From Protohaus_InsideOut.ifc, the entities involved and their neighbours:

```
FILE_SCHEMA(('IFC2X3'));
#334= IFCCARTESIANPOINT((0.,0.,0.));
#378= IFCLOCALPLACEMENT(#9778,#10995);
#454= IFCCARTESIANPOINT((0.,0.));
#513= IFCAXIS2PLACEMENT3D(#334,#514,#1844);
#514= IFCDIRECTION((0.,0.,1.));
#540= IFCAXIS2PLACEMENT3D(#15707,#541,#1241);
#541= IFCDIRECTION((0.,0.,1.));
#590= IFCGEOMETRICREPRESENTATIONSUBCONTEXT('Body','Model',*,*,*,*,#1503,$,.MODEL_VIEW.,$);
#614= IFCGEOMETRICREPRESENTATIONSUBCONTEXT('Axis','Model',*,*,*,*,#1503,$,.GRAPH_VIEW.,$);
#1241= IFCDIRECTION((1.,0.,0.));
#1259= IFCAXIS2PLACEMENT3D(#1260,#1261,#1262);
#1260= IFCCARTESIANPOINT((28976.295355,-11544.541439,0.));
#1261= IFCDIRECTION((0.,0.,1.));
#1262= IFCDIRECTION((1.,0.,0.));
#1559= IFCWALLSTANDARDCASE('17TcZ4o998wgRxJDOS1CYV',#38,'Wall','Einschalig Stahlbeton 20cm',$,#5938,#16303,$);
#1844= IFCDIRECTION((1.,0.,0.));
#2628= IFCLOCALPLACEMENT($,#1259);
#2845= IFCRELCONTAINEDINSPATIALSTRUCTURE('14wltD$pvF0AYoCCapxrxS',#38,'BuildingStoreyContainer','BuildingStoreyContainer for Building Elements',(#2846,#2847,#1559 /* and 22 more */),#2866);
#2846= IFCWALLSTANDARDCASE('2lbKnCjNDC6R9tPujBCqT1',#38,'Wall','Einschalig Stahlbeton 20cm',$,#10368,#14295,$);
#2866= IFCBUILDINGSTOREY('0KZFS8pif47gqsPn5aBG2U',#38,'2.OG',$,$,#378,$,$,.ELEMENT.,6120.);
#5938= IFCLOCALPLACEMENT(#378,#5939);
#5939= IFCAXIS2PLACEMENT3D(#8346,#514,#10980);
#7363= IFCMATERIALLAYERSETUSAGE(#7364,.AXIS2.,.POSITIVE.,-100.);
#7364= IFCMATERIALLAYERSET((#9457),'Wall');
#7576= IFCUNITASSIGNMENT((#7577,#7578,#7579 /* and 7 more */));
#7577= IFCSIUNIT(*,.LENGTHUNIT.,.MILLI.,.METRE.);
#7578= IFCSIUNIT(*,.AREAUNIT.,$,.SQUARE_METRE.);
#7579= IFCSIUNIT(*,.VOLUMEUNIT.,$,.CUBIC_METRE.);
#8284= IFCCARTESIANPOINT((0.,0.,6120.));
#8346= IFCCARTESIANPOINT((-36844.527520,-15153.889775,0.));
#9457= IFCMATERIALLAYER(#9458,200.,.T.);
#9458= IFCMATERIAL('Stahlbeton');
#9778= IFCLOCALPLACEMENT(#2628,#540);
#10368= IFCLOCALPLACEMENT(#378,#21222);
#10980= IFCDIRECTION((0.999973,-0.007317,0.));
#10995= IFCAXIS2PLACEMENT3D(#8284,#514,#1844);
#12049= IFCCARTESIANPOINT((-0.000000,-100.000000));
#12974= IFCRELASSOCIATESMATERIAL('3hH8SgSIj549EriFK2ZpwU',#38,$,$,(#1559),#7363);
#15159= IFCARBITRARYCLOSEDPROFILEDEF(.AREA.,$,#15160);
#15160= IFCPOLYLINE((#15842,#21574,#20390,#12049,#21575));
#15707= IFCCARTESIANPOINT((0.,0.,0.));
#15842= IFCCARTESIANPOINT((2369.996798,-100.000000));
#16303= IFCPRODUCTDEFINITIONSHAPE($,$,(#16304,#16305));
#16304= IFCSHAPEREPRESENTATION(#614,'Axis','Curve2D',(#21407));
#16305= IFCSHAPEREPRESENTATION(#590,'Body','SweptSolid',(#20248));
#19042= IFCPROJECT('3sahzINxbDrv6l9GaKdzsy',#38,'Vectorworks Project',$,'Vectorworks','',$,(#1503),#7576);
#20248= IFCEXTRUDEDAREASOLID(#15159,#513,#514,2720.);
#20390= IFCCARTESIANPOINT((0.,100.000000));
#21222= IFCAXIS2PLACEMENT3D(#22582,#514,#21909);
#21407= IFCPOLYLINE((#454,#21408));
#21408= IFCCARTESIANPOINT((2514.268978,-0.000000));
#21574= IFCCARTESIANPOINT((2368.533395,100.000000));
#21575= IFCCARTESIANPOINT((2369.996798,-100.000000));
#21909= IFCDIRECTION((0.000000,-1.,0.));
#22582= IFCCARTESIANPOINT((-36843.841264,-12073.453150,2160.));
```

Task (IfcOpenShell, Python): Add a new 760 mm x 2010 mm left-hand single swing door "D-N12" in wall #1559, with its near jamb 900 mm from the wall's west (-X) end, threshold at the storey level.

```python
import numpy as np
import ifcopenshell
import ifcopenshell.api.feature
import ifcopenshell.api.geometry
import ifcopenshell.api.root
import ifcopenshell.api.spatial
import ifcopenshell.api.type
import ifcopenshell.geom
import ifcopenshell.util.element
import ifcopenshell.util.placement
import ifcopenshell.util.representation
import ifcopenshell.util.shape
import ifcopenshell.util.unit

model = ifcopenshell.open("Protohaus_InsideOut.ifc")
unit_scale = ifcopenshell.util.unit.calculate_unit_scale(model)
settings = ifcopenshell.geom.settings()


def volume(element):
    """Net volume in cubic metres, openings subtracted."""
    shape = ifcopenshell.geom.create_shape(settings, element)
    return ifcopenshell.util.shape.get_volume(shape.geometry)


wall = model.by_guid("17TcZ4o998wgRxJDOS1CYV")
storey = ifcopenshell.util.element.get_container(wall, ifc_class="IfcBuildingStorey")
context = ifcopenshell.util.representation.get_context(model, "Model", "Body", "MODEL_VIEW")
before = volume(wall)

width, height, from_end, sill = 0.76, 2.01, 0.9, 0.0  # metres

# The wall runs along its own X axis, and the end named is its -X end.
wall_shape = ifcopenshell.geom.create_shape(settings, wall)
x, y, z = ifcopenshell.util.shape.get_vertices(wall_shape.geometry).T
start = x.min() + from_end
face, thickness = float(y.min()), float(y.max() - y.min())
wall_matrix = ifcopenshell.util.placement.get_local_placement(wall.ObjectPlacement)
level = ifcopenshell.util.placement.get_local_placement(storey.ObjectPlacement)[2, 3]


def in_wall(x, y):
    """Placement at x, y metres in the wall's axes, at sill height."""
    matrix = wall_matrix.copy()
    matrix[:, 3] = wall_matrix @ np.array([x / unit_scale, y / unit_scale, 0.0, 1.0])
    matrix[2, 3] = level + sill / unit_scale
    return matrix


# Opening: a box that overshoots both wall faces by 50 mm.
opening = ifcopenshell.api.root.create_entity(model, ifc_class="IfcOpeningElement")
box = ifcopenshell.api.geometry.add_wall_representation(
    model, context=context, length=width, height=height, thickness=thickness + 0.1
)
ifcopenshell.api.geometry.assign_representation(model, product=opening, representation=box)
ifcopenshell.api.geometry.edit_object_placement(model, product=opening, matrix=in_wall(start, face - 0.05), is_si=False)
ifcopenshell.api.feature.add_feature(model, feature=opening, element=wall)

door = ifcopenshell.api.root.create_entity(model, ifc_class="IfcDoor", name="D-N12")
door.OverallWidth, door.OverallHeight = width / unit_scale, height / unit_scale
body = ifcopenshell.api.geometry.add_door_representation(
    model,
    context=context,
    overall_width=door.OverallWidth,
    overall_height=door.OverallHeight,
    operation_type="SINGLE_SWING_LEFT",
    lining_properties={"LiningDepth": thickness / unit_scale, "ThresholdDepth": thickness / unit_scale},
)
ifcopenshell.api.geometry.assign_representation(model, product=door, representation=body)
ifcopenshell.api.spatial.assign_container(model, products=[door], relating_structure=storey)
fills = ifcopenshell.api.feature.add_filling(model, opening=opening, element=door)
fills.OwnerHistory = door.OwnerHistory  # required in IFC2X3

# IFC2X3 keeps the operation on the door style.
style = ifcopenshell.api.root.create_entity(model, ifc_class="IfcDoorStyle", name="D-N12")
style.OperationType, style.ConstructionType = "SINGLE_SWING_LEFT", "NOTDEFINED"
style.ParameterTakesPrecedence = style.Sizeable = False
ifcopenshell.api.type.assign_type(model, related_objects=[door], relating_type=style)

# The lining spans the wall, so the door starts at the wall face.
ifcopenshell.api.geometry.edit_object_placement(model, product=door, matrix=in_wall(start, face), is_si=False)

after = volume(wall)

print(f"wall volume {before:.3f} -> {after:.3f} m3")

model.write("Protohaus_InsideOut_rev.ifc")
```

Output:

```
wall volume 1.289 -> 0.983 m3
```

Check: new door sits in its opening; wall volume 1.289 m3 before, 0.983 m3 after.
